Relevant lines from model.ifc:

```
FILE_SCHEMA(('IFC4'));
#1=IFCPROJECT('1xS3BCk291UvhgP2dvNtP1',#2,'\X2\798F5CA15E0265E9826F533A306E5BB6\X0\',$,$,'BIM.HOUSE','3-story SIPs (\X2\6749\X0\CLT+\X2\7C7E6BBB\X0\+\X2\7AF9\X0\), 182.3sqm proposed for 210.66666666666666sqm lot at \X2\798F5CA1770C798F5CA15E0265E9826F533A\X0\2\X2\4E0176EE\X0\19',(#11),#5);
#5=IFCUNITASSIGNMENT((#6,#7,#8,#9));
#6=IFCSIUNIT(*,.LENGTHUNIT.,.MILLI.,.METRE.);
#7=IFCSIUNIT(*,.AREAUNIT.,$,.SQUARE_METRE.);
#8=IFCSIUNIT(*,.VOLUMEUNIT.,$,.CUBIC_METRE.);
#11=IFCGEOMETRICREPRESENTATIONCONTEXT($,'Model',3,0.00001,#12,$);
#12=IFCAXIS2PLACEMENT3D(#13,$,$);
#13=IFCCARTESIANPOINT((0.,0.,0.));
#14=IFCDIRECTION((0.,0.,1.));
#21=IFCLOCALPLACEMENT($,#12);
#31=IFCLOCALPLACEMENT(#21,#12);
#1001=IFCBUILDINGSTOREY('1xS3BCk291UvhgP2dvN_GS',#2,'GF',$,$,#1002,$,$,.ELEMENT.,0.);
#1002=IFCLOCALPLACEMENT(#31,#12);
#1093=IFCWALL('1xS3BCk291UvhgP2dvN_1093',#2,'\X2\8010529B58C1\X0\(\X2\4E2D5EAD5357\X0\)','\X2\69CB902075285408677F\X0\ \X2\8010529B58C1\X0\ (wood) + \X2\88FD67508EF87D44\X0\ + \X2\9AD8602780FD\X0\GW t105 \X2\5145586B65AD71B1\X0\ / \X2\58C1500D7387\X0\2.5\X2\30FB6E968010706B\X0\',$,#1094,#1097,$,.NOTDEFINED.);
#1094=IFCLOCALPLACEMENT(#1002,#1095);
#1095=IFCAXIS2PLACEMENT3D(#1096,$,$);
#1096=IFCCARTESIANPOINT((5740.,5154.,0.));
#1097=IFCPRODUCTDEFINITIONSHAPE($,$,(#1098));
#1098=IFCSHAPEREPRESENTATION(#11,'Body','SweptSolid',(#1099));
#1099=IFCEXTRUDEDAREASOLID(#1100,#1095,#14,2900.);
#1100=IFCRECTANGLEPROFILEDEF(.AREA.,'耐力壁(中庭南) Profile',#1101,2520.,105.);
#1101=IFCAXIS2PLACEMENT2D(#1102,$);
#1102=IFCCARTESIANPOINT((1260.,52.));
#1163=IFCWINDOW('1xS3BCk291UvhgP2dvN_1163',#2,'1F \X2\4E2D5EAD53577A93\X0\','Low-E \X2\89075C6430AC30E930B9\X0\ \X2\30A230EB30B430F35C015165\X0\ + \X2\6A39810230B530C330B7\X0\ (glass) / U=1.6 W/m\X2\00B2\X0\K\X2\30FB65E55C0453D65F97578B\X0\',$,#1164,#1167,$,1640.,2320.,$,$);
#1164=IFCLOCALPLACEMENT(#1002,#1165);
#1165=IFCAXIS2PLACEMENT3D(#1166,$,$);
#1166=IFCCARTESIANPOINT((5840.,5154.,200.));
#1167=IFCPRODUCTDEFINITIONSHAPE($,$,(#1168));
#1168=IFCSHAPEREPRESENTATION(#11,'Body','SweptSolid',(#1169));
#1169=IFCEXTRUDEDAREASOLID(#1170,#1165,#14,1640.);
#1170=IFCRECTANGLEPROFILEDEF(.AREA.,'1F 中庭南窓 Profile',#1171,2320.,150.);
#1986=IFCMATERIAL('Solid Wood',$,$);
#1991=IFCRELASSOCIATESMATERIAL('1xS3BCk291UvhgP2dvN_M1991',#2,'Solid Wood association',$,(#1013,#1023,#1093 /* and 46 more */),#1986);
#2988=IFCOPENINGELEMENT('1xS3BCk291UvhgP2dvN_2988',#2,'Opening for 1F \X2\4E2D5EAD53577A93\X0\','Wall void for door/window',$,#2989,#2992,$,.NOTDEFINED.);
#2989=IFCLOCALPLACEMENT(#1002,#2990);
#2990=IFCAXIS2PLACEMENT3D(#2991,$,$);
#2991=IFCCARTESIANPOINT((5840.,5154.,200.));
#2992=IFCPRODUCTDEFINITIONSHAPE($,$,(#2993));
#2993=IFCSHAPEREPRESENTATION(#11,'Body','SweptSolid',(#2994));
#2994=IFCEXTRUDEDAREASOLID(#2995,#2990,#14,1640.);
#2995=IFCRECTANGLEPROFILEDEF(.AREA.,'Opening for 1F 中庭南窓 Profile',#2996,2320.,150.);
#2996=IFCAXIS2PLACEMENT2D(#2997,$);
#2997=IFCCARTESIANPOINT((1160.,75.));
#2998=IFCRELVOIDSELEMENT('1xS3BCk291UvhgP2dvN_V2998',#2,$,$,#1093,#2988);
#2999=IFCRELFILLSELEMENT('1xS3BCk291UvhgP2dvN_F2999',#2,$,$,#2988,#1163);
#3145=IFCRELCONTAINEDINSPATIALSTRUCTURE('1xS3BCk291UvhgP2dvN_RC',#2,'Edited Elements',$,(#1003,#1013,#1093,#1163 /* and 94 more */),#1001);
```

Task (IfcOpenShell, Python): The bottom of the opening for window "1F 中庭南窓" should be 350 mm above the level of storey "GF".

```python
import numpy as np
import ifcopenshell
import ifcopenshell.api.geometry
import ifcopenshell.geom
import ifcopenshell.util.element
import ifcopenshell.util.placement
import ifcopenshell.util.shape
import ifcopenshell.util.unit

model = ifcopenshell.open("model.ifc")
unit_scale = ifcopenshell.util.unit.calculate_unit_scale(model)

window = model.by_guid("1xS3BCk291UvhgP2dvN_1163")
opening = window.FillsVoids[0].RelatingOpeningElement
storey = ifcopenshell.util.element.get_container(window, ifc_class="IfcBuildingStorey")
level = ifcopenshell.util.placement.get_local_placement(storey.ObjectPlacement)[2, 3]

# The opening's origin need not be at the sill, so measure its lowest point.
shape = ifcopenshell.geom.create_shape(ifcopenshell.geom.settings(), opening)
bottom = ifcopenshell.util.shape.get_shape_bottom_elevation(shape, shape.geometry) / unit_scale
dz = level + 0.35 / unit_scale - bottom

shift = np.array([0.0, 0.0, dz])
# The window is not placed relative to its opening, so move both.
for product in (opening, window):
    matrix = ifcopenshell.util.placement.get_local_placement(product.ObjectPlacement)
    matrix[:3, 3] += shift
    ifcopenshell.api.geometry.edit_object_placement(model, product=product, matrix=matrix, is_si=False)

print(f"moved by {dz * unit_scale:+.3f} m")

model.write("model_v2.ifc")
```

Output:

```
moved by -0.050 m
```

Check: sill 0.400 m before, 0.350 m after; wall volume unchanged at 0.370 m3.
